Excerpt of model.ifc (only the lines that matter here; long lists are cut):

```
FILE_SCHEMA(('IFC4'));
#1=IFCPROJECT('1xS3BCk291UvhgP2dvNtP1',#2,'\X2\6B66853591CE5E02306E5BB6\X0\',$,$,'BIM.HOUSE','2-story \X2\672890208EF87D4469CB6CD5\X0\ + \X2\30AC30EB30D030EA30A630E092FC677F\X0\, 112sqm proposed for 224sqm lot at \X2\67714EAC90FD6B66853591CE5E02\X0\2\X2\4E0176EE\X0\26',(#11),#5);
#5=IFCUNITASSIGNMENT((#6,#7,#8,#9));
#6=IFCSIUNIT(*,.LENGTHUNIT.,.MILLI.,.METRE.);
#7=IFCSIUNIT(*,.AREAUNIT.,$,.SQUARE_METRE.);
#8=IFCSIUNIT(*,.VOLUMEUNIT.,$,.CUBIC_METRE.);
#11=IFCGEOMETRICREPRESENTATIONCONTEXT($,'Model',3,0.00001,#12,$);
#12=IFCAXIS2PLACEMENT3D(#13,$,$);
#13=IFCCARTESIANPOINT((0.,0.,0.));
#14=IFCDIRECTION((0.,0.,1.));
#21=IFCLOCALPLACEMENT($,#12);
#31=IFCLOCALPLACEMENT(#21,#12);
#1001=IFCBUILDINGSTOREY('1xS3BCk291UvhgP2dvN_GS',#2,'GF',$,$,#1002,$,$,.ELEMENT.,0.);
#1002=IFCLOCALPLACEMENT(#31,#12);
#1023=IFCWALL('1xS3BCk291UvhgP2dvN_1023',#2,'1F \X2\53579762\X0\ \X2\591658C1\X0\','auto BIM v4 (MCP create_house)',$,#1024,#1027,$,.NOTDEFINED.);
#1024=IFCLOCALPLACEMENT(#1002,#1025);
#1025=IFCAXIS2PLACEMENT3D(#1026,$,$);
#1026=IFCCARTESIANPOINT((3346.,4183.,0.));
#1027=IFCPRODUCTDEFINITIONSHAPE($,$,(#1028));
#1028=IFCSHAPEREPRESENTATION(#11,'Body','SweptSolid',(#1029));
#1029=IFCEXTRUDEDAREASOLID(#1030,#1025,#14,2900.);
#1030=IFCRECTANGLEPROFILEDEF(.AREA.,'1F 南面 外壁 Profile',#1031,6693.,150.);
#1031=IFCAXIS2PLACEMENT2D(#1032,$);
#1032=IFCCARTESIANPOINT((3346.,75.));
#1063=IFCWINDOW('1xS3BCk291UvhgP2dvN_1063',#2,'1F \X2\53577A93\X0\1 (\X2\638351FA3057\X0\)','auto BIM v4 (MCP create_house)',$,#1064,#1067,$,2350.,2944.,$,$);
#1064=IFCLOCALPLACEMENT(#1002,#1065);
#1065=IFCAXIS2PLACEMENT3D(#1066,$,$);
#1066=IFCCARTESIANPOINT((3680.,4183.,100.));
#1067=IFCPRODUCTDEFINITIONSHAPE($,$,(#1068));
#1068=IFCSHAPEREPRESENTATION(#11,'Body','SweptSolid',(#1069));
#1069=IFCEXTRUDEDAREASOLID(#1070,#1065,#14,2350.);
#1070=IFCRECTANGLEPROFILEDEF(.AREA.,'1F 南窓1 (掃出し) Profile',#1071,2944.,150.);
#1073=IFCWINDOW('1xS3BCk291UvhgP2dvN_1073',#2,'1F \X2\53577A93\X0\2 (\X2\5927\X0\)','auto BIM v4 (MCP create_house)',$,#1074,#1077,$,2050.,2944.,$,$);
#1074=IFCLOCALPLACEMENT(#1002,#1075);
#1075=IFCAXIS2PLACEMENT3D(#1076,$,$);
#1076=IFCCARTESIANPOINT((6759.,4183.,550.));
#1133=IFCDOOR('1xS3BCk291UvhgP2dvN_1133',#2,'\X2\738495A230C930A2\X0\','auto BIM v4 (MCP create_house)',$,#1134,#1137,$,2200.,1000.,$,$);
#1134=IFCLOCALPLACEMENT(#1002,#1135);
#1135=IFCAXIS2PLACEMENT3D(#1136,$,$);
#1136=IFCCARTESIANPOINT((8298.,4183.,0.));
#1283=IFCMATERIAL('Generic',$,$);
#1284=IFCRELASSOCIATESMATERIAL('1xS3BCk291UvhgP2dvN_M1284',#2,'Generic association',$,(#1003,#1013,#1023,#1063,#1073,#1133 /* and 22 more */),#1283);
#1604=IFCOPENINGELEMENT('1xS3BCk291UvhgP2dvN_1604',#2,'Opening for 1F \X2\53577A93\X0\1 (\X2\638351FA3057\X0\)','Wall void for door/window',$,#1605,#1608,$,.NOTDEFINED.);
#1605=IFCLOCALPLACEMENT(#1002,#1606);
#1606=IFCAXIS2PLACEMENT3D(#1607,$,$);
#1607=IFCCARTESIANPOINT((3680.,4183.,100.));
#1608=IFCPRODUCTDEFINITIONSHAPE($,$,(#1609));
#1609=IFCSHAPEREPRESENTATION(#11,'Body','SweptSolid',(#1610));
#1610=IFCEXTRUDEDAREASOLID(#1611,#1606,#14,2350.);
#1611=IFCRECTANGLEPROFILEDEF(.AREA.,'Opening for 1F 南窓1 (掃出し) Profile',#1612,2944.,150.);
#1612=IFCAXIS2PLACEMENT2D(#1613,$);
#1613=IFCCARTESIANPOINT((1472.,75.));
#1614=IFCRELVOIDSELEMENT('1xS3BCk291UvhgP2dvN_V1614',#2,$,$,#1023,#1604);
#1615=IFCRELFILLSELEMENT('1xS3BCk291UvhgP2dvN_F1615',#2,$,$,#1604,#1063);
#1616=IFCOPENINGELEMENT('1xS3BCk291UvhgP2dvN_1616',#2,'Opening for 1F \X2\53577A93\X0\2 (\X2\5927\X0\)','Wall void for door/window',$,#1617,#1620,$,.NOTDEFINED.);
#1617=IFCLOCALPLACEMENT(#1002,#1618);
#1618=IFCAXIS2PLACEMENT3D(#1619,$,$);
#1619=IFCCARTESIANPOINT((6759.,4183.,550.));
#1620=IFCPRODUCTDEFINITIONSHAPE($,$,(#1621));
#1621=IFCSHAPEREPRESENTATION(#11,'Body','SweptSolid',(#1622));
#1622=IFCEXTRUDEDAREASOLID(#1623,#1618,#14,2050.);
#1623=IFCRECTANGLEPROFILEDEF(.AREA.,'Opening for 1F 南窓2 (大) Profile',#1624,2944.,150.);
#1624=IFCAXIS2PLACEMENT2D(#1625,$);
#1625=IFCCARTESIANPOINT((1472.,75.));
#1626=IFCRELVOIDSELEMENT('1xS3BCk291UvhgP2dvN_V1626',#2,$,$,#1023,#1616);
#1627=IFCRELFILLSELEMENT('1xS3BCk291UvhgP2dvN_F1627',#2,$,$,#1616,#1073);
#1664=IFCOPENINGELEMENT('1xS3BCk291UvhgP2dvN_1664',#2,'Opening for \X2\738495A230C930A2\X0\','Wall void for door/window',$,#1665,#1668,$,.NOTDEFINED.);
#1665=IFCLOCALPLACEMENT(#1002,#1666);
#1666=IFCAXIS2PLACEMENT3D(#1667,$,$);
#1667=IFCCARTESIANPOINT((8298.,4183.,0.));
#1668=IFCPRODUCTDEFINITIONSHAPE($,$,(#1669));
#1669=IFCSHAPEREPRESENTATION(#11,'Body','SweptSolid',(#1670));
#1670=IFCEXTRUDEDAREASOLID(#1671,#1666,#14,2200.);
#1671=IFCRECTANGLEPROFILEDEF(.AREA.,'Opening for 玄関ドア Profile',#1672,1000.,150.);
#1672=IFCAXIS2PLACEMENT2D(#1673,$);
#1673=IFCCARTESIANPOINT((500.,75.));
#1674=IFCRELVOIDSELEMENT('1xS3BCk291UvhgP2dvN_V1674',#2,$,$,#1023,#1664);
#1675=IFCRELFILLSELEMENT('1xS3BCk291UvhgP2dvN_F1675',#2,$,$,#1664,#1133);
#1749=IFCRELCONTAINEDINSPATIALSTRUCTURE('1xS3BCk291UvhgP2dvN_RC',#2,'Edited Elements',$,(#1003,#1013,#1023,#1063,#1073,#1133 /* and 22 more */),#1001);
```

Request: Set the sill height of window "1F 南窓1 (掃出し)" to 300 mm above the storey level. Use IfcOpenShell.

```python
import numpy as np
import ifcopenshell
import ifcopenshell.api.geometry
import ifcopenshell.geom
import ifcopenshell.util.element
import ifcopenshell.util.placement
import ifcopenshell.util.shape
import ifcopenshell.util.unit

model = ifcopenshell.open("model.ifc")
unit_scale = ifcopenshell.util.unit.calculate_unit_scale(model)

window = model.by_guid("1xS3BCk291UvhgP2dvN_1063")
opening = window.FillsVoids[0].RelatingOpeningElement
storey = ifcopenshell.util.element.get_container(window, ifc_class="IfcBuildingStorey")
level = ifcopenshell.util.placement.get_local_placement(storey.ObjectPlacement)[2, 3]

# The opening's origin need not be at the sill, so measure its lowest point.
shape = ifcopenshell.geom.create_shape(ifcopenshell.geom.settings(), opening)
bottom = ifcopenshell.util.shape.get_shape_bottom_elevation(shape, shape.geometry) / unit_scale
dz = level + 0.3 / unit_scale - bottom

shift = np.array([0.0, 0.0, dz])
# The window is not placed relative to its opening, so move both.
for product in (opening, window):
    matrix = ifcopenshell.util.placement.get_local_placement(product.ObjectPlacement)
    matrix[:3, 3] += shift
    ifcopenshell.api.geometry.edit_object_placement(model, product=product, matrix=matrix, is_si=False)

print(f"moved by {dz * unit_scale:+.3f} m")

model.write("model_updated.ifc")
```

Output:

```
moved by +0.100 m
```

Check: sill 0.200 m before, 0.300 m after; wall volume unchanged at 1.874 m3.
